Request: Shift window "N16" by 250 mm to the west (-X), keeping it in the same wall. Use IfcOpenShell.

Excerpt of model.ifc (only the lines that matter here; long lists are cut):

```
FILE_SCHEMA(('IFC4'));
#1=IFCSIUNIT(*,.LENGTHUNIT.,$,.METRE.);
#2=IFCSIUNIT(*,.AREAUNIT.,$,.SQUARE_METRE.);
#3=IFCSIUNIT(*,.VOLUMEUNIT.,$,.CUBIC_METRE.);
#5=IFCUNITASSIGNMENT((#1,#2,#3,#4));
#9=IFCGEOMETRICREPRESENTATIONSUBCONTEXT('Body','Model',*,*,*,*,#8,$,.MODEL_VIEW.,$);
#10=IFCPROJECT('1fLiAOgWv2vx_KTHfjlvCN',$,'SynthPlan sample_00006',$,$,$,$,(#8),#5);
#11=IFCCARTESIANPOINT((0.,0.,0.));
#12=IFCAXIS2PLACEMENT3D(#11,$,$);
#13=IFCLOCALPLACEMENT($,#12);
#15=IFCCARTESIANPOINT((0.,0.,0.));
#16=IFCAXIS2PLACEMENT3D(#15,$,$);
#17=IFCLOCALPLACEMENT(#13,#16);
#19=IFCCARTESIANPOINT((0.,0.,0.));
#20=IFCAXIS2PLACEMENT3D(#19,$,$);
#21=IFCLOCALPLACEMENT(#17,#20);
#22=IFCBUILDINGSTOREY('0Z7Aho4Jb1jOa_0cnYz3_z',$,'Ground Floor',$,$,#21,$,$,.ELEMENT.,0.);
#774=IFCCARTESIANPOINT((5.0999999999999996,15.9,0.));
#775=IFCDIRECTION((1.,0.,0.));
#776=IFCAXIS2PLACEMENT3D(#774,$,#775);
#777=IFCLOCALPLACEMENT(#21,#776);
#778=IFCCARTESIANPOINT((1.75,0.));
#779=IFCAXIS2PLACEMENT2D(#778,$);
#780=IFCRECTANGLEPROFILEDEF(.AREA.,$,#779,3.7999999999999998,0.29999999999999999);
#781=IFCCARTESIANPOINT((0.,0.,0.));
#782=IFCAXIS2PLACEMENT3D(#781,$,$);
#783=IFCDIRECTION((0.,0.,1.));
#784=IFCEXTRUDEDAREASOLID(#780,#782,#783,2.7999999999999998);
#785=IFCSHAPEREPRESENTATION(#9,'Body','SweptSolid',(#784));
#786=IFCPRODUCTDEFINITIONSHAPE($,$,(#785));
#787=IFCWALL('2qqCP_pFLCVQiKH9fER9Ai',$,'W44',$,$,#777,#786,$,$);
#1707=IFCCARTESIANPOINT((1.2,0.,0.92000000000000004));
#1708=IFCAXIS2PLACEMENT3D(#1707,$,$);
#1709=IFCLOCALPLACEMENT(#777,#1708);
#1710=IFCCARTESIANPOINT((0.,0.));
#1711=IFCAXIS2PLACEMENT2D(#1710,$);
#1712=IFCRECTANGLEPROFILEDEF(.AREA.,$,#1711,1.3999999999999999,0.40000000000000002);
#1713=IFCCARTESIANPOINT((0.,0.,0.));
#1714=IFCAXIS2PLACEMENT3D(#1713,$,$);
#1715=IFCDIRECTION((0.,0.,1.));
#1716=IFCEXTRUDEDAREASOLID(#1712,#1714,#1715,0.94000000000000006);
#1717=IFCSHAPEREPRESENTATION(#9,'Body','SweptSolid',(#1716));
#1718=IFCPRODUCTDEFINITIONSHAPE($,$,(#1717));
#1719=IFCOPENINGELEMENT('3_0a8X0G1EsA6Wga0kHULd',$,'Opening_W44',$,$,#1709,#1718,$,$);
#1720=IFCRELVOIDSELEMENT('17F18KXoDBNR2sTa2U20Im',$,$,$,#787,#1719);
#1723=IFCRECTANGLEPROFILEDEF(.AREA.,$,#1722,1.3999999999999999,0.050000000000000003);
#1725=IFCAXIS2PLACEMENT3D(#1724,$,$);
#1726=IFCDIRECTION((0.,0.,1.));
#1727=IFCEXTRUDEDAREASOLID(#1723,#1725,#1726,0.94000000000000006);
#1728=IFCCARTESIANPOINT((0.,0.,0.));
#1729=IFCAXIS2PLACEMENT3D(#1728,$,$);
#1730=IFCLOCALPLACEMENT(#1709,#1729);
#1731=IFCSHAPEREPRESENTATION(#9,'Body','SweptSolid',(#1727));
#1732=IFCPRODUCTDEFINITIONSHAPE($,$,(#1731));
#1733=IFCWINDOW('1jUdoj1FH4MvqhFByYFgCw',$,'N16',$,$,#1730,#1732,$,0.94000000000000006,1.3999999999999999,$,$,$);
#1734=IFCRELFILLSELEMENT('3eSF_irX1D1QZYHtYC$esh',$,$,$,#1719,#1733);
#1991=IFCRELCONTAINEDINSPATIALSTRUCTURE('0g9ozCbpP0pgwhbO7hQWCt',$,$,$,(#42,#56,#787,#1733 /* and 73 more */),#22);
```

```python
import ifcopenshell
import ifcopenshell.api.geometry
import ifcopenshell.util.placement

model = ifcopenshell.open("model.ifc")

window = model.by_id(1733)
opening = window.FillsVoids[0].RelatingOpeningElement
wall = opening.VoidsElements[0].RelatingBuildingElement

wall_matrix = ifcopenshell.util.placement.get_local_placement(wall.ObjectPlacement)
shift = wall_matrix[:3, 0] * -0.25
before = ifcopenshell.util.placement.get_local_placement(window.ObjectPlacement)[:3, 3].copy()

# The window is placed relative to its opening, so it follows when the opening moves.
matrix = ifcopenshell.util.placement.get_local_placement(opening.ObjectPlacement)
matrix[:3, 3] += shift
ifcopenshell.api.geometry.edit_object_placement(
    model, product=opening, matrix=matrix, is_si=False, should_transform_children=True
)

after = ifcopenshell.util.placement.get_local_placement(window.ObjectPlacement)[:3, 3]
print("window moved by", (after - before).round(3) + 0.0)

model.write("model_rev.ifc")
```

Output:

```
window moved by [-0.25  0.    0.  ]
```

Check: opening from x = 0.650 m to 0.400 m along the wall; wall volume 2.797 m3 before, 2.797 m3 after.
